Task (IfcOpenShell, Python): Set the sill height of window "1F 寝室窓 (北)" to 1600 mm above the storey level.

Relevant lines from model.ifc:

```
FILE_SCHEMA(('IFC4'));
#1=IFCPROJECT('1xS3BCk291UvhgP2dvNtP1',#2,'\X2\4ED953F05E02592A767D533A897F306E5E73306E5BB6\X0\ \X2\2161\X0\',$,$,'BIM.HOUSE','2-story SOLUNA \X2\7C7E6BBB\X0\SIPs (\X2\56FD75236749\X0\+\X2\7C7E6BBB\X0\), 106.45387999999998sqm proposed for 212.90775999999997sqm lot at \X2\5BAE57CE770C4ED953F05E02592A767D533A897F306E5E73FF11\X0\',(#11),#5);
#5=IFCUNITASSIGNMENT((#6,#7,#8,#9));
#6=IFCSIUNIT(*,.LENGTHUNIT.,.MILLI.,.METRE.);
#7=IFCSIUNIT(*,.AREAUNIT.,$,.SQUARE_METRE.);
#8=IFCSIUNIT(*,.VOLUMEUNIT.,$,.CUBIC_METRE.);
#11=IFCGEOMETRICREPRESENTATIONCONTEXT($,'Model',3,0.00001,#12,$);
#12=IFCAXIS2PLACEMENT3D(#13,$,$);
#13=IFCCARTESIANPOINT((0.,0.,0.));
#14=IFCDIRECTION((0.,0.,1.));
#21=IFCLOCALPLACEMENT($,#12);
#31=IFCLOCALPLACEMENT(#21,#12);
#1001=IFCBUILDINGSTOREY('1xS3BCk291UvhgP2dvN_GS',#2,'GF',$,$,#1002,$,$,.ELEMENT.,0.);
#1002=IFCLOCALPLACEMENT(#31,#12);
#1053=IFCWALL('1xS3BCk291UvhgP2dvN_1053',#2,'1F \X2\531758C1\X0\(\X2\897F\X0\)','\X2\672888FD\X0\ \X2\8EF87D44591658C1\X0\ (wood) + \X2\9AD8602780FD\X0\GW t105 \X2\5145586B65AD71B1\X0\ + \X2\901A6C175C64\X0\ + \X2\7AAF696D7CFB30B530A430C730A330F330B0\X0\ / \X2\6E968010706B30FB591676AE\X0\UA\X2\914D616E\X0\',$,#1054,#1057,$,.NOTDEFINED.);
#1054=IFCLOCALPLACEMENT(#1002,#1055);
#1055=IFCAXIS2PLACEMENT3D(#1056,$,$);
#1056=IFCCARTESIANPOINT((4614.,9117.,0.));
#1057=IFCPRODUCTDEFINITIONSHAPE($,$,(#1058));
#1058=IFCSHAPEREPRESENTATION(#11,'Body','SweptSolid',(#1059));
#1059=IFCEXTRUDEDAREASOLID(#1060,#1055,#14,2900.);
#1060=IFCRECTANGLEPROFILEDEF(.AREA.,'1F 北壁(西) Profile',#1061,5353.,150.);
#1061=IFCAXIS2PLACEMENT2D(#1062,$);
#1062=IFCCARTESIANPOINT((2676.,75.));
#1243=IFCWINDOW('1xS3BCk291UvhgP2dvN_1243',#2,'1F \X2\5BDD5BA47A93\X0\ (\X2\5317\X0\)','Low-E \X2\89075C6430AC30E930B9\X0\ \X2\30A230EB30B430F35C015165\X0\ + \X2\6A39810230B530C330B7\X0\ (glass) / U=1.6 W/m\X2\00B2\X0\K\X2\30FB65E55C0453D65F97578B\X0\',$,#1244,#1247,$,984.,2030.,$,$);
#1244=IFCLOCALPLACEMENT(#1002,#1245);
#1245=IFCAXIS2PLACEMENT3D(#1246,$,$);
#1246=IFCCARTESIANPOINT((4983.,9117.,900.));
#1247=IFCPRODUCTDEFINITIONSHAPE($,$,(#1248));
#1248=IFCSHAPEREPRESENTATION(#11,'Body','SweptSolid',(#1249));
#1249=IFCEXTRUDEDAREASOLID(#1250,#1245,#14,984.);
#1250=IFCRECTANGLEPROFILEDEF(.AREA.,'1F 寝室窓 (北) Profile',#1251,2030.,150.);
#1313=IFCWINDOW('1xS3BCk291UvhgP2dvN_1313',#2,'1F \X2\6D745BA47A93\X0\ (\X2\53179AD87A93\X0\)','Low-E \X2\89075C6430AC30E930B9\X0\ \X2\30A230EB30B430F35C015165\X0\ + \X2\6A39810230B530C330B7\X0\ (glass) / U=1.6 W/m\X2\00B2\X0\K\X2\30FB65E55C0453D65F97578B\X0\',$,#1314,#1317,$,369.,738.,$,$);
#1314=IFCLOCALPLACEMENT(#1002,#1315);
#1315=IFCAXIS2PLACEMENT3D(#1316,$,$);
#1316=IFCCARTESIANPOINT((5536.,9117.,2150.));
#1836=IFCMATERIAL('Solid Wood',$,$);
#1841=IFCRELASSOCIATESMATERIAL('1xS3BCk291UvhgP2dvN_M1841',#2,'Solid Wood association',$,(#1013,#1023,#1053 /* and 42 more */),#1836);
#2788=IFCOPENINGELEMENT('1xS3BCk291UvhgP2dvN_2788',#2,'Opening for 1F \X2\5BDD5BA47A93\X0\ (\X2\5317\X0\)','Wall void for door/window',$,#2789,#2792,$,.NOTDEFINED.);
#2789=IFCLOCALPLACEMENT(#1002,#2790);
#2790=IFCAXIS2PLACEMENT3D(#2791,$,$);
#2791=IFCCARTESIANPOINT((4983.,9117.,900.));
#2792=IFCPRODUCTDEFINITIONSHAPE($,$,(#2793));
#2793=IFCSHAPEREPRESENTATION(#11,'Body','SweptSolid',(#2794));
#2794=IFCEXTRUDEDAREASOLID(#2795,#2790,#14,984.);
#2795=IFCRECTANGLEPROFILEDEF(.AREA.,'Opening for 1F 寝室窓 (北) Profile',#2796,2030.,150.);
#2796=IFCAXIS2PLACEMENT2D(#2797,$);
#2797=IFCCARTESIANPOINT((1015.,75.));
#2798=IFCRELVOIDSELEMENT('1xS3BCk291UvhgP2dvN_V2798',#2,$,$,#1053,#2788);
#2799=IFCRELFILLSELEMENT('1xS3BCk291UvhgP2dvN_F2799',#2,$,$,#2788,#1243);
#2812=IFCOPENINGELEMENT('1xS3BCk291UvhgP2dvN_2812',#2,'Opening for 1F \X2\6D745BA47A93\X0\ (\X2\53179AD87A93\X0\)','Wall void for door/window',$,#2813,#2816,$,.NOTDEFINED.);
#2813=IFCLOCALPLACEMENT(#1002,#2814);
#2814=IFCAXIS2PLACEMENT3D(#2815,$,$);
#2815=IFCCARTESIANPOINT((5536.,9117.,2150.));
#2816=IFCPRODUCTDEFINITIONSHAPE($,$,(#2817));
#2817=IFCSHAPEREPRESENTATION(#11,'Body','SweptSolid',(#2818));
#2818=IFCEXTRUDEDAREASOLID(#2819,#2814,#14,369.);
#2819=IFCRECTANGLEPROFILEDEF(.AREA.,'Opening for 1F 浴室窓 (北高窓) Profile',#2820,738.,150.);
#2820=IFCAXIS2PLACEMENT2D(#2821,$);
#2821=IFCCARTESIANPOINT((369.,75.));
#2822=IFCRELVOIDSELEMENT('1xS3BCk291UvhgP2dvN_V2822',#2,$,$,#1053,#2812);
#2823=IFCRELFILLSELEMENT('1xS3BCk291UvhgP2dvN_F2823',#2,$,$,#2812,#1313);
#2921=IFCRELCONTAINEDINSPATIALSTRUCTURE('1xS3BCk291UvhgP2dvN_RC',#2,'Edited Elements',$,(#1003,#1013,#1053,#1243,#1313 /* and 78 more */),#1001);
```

```python
import numpy as np
import ifcopenshell
import ifcopenshell.api.geometry
import ifcopenshell.geom
import ifcopenshell.util.element
import ifcopenshell.util.placement
import ifcopenshell.util.shape
import ifcopenshell.util.unit

model = ifcopenshell.open("model.ifc")
unit_scale = ifcopenshell.util.unit.calculate_unit_scale(model)

window = model.by_id(1243)
opening = window.FillsVoids[0].RelatingOpeningElement
storey = ifcopenshell.util.element.get_container(window, ifc_class="IfcBuildingStorey")
level = ifcopenshell.util.placement.get_local_placement(storey.ObjectPlacement)[2, 3]

# The opening's origin need not be at the sill, so measure its lowest point.
shape = ifcopenshell.geom.create_shape(ifcopenshell.geom.settings(), opening)
bottom = ifcopenshell.util.shape.get_shape_bottom_elevation(shape, shape.geometry) / unit_scale
dz = level + 1.6 / unit_scale - bottom

shift = np.array([0.0, 0.0, dz])
# The window is not placed relative to its opening, so move both.
for product in (opening, window):
    matrix = ifcopenshell.util.placement.get_local_placement(product.ObjectPlacement)
    matrix[:3, 3] += shift
    ifcopenshell.api.geometry.edit_object_placement(model, product=product, matrix=matrix, is_si=False)

print(f"moved by {dz * unit_scale:+.3f} m")

model.write("model_updated.ifc")
```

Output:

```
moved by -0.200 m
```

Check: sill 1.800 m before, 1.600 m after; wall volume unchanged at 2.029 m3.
